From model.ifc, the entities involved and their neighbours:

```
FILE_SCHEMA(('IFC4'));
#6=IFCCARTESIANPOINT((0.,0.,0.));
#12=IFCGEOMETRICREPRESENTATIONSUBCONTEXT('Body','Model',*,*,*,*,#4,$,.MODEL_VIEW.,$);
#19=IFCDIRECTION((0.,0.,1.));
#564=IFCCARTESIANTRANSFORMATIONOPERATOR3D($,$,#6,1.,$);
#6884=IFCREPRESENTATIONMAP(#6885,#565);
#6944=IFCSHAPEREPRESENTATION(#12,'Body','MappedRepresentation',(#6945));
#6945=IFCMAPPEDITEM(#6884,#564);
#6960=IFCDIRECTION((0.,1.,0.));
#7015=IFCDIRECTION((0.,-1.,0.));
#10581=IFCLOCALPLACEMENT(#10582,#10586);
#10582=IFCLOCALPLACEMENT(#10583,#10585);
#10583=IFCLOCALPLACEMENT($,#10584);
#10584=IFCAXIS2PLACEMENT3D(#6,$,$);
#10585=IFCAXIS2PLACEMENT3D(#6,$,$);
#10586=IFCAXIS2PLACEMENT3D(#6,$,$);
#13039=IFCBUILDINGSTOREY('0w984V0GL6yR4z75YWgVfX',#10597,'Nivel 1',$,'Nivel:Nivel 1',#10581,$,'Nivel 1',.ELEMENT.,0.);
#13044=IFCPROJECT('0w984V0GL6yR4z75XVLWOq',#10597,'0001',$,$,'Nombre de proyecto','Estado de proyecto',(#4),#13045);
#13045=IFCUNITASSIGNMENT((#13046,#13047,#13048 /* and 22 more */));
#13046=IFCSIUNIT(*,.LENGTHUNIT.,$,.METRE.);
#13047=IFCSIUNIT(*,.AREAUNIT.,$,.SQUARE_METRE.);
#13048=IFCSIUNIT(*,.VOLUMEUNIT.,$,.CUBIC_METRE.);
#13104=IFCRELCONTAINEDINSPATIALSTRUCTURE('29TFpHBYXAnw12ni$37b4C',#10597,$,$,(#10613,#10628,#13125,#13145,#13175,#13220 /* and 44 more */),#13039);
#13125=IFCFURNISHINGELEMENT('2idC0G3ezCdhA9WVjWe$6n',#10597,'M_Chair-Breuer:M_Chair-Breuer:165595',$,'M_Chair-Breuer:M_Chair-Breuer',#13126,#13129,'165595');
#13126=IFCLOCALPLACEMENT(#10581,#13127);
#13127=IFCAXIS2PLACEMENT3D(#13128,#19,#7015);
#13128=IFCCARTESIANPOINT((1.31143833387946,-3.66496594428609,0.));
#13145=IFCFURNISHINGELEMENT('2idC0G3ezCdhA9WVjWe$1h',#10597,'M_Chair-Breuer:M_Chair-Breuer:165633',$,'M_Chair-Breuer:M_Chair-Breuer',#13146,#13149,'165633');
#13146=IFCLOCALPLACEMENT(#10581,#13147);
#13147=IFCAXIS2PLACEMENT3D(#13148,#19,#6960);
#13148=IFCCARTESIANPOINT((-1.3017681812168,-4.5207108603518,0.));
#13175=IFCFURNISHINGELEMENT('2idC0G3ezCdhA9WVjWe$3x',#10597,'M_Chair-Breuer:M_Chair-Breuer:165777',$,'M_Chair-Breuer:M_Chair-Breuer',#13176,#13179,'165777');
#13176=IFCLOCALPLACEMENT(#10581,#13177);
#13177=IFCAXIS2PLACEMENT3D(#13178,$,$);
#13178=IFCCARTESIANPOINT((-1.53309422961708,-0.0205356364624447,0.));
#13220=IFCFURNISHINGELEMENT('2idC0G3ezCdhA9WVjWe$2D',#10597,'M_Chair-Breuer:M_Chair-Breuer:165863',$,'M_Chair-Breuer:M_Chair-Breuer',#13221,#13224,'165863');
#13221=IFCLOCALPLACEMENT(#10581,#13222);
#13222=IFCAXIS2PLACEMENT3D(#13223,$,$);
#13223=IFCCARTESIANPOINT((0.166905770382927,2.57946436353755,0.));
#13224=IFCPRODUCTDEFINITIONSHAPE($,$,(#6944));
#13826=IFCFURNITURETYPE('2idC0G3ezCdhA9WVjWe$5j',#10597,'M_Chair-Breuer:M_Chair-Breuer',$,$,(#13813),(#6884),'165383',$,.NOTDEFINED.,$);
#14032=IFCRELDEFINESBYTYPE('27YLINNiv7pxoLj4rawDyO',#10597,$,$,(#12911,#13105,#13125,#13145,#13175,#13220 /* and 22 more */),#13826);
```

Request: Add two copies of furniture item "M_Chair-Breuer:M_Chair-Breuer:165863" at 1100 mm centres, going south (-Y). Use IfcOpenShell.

```python
import numpy as np
import ifcopenshell
import ifcopenshell.api.geometry
import ifcopenshell.api.root
import ifcopenshell.util.element
import ifcopenshell.util.placement

model = ifcopenshell.open("model.ifc")


def reuse_history(source, copy):
    """copy_class also copies each property set's owner history, people and application; keep the originals."""
    for rel in copy.IsDefinedBy:
        if rel.is_a("IfcRelDefinesByProperties") and (history := rel.RelatingPropertyDefinition.OwnerHistory):
            rel.RelatingPropertyDefinition.OwnerHistory = source.OwnerHistory
            ifcopenshell.util.element.remove_deep2(model, history)


source = model.by_id(13220)
base = ifcopenshell.util.placement.get_local_placement(source.ObjectPlacement)
step = np.array([0.0, -1.0, 0.0]) * 1.1

for i in range(1, 3):
    copy = ifcopenshell.api.root.copy_class(model, product=source)
    copy.Representation = ifcopenshell.util.element.copy_deep(
        model, source.Representation, exclude=["IfcGeometricRepresentationContext", "IfcRepresentationMap"]
    )
    copy.Name = "M_Chair-Breuer:M_Chair-Breuer"
    copy.Tag = None
    reuse_history(source, copy)
    matrix = base.copy()
    matrix[:3, 3] += i * step
    print("added at", matrix[:3, 3].round(3) + 0.0)
    ifcopenshell.api.geometry.edit_object_placement(model, product=copy, matrix=matrix, is_si=False)

model.write("model-out.ifc")
```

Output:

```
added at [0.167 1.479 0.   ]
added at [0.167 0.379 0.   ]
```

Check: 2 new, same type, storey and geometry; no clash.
